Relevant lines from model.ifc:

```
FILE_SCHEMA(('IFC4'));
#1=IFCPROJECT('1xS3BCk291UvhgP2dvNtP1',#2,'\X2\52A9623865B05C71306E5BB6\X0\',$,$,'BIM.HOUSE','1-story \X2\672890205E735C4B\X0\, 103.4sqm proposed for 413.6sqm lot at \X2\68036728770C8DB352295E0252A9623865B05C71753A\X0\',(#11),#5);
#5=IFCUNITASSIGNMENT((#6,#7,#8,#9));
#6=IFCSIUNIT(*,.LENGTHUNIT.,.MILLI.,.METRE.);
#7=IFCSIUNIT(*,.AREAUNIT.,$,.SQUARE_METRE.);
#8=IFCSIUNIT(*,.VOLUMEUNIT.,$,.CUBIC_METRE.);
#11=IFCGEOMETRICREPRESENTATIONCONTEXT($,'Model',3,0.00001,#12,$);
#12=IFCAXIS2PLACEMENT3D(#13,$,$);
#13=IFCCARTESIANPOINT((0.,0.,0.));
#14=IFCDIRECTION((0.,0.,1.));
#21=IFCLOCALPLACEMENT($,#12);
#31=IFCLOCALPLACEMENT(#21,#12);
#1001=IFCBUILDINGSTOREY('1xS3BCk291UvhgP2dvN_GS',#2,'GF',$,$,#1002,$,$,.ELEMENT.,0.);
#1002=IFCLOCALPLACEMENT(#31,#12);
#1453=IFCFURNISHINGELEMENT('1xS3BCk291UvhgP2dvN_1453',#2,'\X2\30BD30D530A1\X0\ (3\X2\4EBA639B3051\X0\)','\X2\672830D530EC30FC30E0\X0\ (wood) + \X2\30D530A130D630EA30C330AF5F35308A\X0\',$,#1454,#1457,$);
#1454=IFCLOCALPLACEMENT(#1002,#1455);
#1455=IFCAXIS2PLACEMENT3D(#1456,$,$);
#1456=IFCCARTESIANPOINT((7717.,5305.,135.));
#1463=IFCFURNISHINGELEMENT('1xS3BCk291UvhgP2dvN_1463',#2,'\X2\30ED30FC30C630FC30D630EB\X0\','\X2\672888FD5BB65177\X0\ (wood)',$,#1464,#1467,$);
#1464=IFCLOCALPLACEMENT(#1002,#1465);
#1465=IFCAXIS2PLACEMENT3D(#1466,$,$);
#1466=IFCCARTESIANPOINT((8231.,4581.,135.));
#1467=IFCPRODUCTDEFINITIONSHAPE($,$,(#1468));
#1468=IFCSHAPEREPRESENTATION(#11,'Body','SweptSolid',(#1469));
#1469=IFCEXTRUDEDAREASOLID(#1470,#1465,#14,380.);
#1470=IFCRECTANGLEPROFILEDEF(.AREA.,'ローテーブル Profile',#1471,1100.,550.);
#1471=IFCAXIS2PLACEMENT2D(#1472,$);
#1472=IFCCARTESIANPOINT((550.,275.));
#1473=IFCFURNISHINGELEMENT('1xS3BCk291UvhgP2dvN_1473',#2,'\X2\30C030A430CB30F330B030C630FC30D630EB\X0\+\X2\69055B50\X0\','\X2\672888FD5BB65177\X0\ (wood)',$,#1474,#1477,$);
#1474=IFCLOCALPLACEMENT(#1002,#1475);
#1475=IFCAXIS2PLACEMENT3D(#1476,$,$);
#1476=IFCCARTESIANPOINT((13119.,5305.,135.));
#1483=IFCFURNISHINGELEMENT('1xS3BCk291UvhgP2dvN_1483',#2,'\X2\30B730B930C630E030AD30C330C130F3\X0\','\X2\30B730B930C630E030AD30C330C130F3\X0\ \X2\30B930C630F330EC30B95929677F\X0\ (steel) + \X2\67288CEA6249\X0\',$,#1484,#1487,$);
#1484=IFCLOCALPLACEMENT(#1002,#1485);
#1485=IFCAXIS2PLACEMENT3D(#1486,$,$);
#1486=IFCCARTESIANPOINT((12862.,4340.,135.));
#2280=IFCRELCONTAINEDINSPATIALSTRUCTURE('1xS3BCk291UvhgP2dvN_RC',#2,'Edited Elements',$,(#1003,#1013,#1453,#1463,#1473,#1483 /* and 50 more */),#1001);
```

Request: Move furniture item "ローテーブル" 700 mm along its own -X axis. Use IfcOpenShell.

```python
import ifcopenshell
import ifcopenshell.api.geometry
import ifcopenshell.util.placement
import ifcopenshell.util.unit

model = ifcopenshell.open("model.ifc")
unit_scale = ifcopenshell.util.unit.calculate_unit_scale(model)

item = model.by_id(1463)
matrix = ifcopenshell.util.placement.get_local_placement(item.ObjectPlacement)
matrix[:3, 3] -= matrix[:3, 0] * 0.7 / unit_scale
ifcopenshell.api.geometry.edit_object_placement(model, product=item, matrix=matrix, is_si=False)

print(ifcopenshell.util.placement.get_local_placement(item.ObjectPlacement).round(3) + 0.0)

model.write("model_updated.ifc")
```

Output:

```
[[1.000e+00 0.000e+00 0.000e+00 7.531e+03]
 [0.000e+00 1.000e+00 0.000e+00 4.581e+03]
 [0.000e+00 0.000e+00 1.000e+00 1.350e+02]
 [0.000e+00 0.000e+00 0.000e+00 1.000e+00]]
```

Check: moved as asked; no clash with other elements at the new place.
